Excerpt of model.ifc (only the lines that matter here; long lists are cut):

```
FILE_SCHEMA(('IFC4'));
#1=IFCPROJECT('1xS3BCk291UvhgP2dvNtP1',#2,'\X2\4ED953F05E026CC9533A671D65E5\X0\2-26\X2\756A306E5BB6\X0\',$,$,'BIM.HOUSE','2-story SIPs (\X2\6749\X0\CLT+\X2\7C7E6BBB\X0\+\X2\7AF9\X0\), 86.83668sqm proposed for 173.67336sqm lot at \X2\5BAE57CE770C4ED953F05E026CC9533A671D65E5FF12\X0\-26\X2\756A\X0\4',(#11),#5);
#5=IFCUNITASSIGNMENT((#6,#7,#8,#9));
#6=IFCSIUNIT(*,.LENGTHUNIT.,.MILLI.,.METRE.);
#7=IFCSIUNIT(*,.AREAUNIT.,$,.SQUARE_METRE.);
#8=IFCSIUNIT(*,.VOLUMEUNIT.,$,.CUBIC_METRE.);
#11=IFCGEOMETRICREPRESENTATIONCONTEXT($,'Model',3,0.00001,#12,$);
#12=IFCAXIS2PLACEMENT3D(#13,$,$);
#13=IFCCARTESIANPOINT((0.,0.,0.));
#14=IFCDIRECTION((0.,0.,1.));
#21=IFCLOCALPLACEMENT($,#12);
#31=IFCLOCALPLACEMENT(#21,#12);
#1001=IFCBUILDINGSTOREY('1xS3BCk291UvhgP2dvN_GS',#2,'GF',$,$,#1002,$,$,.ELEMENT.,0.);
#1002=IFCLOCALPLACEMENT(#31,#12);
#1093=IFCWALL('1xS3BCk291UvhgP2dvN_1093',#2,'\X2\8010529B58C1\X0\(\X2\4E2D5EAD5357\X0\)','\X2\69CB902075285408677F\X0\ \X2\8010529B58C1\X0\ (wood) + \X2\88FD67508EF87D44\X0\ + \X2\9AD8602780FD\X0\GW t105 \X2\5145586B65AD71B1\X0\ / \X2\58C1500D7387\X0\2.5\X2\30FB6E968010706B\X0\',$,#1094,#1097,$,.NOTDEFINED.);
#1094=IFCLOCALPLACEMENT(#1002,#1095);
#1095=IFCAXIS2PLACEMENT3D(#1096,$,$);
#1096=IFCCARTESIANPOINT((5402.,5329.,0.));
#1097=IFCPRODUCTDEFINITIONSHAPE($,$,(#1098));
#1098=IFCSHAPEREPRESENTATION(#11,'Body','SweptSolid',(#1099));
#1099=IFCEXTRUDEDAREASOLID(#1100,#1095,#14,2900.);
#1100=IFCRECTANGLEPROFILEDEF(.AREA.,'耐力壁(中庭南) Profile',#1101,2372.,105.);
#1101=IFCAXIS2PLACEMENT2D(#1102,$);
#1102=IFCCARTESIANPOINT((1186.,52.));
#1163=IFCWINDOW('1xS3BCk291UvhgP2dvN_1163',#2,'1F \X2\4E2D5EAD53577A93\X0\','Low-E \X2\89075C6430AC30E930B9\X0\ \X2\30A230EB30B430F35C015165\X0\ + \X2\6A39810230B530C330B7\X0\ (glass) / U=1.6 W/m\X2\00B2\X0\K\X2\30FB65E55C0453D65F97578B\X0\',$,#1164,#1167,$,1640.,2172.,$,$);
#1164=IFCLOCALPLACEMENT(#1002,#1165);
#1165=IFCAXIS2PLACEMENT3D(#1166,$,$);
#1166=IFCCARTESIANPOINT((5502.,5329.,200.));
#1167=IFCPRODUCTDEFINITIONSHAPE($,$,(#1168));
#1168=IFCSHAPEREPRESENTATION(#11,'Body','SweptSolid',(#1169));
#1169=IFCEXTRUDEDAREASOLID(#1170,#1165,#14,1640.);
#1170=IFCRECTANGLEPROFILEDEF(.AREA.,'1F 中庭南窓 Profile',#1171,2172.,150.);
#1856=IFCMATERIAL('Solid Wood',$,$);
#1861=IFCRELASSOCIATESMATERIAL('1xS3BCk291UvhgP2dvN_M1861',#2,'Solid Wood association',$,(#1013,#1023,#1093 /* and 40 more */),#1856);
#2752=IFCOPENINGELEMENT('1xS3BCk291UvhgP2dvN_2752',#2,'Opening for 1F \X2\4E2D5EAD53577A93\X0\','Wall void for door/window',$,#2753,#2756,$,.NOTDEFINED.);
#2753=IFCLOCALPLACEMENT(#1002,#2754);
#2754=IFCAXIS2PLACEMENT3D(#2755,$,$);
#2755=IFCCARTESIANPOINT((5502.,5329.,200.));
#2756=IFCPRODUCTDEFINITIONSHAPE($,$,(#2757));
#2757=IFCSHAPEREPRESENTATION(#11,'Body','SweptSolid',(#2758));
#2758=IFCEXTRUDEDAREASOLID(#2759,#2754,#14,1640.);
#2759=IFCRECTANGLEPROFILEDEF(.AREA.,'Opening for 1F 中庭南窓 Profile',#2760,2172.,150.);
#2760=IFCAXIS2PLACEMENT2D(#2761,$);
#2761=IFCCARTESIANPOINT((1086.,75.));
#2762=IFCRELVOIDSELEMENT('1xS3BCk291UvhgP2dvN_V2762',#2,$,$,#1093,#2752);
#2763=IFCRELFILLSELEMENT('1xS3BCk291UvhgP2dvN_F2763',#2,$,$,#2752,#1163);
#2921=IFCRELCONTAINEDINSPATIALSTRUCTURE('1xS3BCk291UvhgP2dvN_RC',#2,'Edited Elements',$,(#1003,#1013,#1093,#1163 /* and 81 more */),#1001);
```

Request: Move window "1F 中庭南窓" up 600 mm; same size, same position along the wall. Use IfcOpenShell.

```python
import numpy as np
import ifcopenshell
import ifcopenshell.api.geometry
import ifcopenshell.util.placement
import ifcopenshell.util.unit

model = ifcopenshell.open("model.ifc")
unit_scale = ifcopenshell.util.unit.calculate_unit_scale(model)

window = model.by_guid("1xS3BCk291UvhgP2dvN_1163")
opening = window.FillsVoids[0].RelatingOpeningElement
dz = 600.0

shift = np.array([0.0, 0.0, dz])
# The window is not placed relative to its opening, so move both.
for product in (opening, window):
    matrix = ifcopenshell.util.placement.get_local_placement(product.ObjectPlacement)
    matrix[:3, 3] += shift
    ifcopenshell.api.geometry.edit_object_placement(model, product=product, matrix=matrix, is_si=False)

print(f"moved by {dz * unit_scale:+.3f} m")

model.write("model_v2.ifc")
```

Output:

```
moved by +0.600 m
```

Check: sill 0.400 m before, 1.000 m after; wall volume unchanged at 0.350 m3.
